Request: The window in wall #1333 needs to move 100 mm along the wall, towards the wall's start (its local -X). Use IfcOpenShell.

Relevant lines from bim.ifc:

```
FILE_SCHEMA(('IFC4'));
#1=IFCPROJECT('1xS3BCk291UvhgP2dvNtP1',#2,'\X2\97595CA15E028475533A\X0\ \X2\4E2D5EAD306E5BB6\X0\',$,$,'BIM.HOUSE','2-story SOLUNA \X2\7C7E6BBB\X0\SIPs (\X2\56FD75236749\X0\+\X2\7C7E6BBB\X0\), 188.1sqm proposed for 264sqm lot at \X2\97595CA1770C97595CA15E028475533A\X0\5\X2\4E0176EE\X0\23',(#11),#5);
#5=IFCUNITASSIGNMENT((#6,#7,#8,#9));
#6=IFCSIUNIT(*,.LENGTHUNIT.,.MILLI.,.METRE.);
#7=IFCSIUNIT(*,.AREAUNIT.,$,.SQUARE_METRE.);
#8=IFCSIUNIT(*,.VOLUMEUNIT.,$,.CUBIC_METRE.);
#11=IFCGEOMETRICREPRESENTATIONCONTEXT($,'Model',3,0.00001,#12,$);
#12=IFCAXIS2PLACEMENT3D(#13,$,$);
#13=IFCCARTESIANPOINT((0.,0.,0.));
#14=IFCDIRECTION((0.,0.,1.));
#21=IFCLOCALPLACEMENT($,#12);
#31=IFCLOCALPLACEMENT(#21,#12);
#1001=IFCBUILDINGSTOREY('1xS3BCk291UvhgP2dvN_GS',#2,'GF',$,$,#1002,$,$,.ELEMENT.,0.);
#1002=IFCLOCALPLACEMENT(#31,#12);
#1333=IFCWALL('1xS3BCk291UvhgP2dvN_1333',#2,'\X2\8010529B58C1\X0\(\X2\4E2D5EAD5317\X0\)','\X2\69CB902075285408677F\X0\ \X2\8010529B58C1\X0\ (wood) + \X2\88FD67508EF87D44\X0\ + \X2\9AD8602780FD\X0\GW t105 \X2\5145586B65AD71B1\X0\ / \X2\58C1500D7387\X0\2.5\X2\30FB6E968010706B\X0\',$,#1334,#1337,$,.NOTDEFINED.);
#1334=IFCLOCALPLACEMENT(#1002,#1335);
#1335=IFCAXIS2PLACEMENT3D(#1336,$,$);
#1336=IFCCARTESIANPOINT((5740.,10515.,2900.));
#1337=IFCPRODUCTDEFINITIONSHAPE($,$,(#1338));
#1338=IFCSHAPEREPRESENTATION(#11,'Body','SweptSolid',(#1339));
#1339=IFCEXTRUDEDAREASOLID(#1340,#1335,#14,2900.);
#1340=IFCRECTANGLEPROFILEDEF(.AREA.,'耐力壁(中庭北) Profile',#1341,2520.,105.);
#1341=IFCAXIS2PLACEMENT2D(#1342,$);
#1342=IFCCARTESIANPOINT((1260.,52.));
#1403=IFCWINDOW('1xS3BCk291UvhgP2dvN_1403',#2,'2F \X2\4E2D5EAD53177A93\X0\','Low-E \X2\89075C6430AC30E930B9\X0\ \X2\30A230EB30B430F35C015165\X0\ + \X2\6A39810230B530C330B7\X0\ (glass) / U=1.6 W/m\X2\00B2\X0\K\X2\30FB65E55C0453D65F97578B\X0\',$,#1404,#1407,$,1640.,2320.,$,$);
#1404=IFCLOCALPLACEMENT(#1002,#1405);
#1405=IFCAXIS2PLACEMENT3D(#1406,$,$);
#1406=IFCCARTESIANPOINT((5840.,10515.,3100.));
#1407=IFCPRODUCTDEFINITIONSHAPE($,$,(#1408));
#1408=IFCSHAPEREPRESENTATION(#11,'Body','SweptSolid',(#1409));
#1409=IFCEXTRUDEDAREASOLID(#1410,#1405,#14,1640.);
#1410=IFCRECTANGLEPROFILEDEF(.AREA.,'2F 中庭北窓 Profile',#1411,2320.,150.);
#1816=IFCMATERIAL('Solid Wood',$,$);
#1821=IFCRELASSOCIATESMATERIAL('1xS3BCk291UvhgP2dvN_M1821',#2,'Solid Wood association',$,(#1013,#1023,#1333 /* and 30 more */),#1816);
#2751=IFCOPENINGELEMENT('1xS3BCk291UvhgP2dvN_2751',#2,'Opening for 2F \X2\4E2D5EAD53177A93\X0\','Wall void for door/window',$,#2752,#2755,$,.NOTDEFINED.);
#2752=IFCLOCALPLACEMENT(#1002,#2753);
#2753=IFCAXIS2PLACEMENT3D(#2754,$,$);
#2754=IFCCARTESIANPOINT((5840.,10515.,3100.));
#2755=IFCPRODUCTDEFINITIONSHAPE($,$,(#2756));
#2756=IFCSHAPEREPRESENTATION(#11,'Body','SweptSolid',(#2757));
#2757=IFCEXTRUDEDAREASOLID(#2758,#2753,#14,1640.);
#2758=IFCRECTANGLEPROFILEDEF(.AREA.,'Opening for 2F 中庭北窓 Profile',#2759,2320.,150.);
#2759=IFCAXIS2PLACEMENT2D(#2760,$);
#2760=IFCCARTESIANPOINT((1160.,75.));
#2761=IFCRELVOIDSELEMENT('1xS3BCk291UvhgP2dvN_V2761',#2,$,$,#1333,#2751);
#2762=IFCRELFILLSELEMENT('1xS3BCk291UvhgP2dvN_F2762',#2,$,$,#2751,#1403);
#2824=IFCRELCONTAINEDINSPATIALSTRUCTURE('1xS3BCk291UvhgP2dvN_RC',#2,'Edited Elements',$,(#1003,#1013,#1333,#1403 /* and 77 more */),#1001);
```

```python
import ifcopenshell
import ifcopenshell.api.geometry
import ifcopenshell.util.placement

model = ifcopenshell.open("bim.ifc")

window = model.by_id(1403)
opening = window.FillsVoids[0].RelatingOpeningElement
wall = opening.VoidsElements[0].RelatingBuildingElement

wall_matrix = ifcopenshell.util.placement.get_local_placement(wall.ObjectPlacement)
shift = wall_matrix[:3, 0] * -100.0
before = ifcopenshell.util.placement.get_local_placement(window.ObjectPlacement)[:3, 3].copy()

# The window is not placed relative to its opening, so move both.
for product in (opening, window):
    matrix = ifcopenshell.util.placement.get_local_placement(product.ObjectPlacement)
    matrix[:3, 3] += shift
    ifcopenshell.api.geometry.edit_object_placement(model, product=product, matrix=matrix, is_si=False)

after = ifcopenshell.util.placement.get_local_placement(window.ObjectPlacement)[:3, 3]
print("window moved by", (after - before).round(3) + 0.0)

model.write("bim-out.ifc")
```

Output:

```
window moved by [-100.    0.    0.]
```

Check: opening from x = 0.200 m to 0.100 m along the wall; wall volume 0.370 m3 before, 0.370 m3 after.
